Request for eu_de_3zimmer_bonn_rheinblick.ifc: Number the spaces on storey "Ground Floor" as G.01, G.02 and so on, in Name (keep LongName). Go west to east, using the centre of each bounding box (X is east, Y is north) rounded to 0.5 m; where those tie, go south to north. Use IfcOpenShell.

First a look at what the model holds.

```python
import ifcopenshell
import ifcopenshell.util.element
import ifcopenshell.util.placement

model = ifcopenshell.open("eu_de_3zimmer_bonn_rheinblick.ifc")
print(model.schema)
storey = next(s for s in model.by_type("IfcBuildingStorey") if s.Name == "Ground Floor")
spaces = [e for e in ifcopenshell.util.element.get_decomposition(storey) if e.is_a("IfcSpace")]
for e in sorted(spaces, key=lambda e: e.id()):
    origin = ifcopenshell.util.placement.get_local_placement(e.ObjectPlacement)[:3, 3]
    print(e.id(), e.Name, e.LongName, origin.round(2) + 0.0, sep=" | ")
```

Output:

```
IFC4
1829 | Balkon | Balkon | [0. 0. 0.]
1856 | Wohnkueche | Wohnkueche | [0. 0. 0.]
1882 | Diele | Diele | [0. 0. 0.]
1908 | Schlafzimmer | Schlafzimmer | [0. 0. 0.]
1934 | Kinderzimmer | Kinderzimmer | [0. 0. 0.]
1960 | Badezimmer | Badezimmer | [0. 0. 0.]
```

```python
import ifcopenshell
import ifcopenshell.geom
import ifcopenshell.util.element
import ifcopenshell.util.shape

model = ifcopenshell.open("eu_de_3zimmer_bonn_rheinblick.ifc")
settings = ifcopenshell.geom.settings()
settings.set("use-world-coords", True)


def centre(element):
    shape = ifcopenshell.geom.create_shape(settings, element)
    return ifcopenshell.util.shape.get_bbox_centroid(shape.geometry)


storey = next(s for s in model.by_type("IfcBuildingStorey") if s.Name == "Ground Floor")
spaces = [e for e in ifcopenshell.util.element.get_decomposition(storey) if e.is_a("IfcSpace")]

# Insertion points can sit at a corner or the storey origin, so sort by the geometry (in metres).
centres = {e: centre(e) for e in spaces}
spaces.sort(key=lambda e: (round(centres[e][0] / 0.5), centres[e][1]))

for i, e in enumerate(spaces, start=1):
    number = f"G.{i:02d}"
    e.Name = number
    print(e.id(), number)

model.write("eu_de_3zimmer_bonn_rheinblick_v2.ifc")
```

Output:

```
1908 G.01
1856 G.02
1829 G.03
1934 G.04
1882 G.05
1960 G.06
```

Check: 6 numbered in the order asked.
